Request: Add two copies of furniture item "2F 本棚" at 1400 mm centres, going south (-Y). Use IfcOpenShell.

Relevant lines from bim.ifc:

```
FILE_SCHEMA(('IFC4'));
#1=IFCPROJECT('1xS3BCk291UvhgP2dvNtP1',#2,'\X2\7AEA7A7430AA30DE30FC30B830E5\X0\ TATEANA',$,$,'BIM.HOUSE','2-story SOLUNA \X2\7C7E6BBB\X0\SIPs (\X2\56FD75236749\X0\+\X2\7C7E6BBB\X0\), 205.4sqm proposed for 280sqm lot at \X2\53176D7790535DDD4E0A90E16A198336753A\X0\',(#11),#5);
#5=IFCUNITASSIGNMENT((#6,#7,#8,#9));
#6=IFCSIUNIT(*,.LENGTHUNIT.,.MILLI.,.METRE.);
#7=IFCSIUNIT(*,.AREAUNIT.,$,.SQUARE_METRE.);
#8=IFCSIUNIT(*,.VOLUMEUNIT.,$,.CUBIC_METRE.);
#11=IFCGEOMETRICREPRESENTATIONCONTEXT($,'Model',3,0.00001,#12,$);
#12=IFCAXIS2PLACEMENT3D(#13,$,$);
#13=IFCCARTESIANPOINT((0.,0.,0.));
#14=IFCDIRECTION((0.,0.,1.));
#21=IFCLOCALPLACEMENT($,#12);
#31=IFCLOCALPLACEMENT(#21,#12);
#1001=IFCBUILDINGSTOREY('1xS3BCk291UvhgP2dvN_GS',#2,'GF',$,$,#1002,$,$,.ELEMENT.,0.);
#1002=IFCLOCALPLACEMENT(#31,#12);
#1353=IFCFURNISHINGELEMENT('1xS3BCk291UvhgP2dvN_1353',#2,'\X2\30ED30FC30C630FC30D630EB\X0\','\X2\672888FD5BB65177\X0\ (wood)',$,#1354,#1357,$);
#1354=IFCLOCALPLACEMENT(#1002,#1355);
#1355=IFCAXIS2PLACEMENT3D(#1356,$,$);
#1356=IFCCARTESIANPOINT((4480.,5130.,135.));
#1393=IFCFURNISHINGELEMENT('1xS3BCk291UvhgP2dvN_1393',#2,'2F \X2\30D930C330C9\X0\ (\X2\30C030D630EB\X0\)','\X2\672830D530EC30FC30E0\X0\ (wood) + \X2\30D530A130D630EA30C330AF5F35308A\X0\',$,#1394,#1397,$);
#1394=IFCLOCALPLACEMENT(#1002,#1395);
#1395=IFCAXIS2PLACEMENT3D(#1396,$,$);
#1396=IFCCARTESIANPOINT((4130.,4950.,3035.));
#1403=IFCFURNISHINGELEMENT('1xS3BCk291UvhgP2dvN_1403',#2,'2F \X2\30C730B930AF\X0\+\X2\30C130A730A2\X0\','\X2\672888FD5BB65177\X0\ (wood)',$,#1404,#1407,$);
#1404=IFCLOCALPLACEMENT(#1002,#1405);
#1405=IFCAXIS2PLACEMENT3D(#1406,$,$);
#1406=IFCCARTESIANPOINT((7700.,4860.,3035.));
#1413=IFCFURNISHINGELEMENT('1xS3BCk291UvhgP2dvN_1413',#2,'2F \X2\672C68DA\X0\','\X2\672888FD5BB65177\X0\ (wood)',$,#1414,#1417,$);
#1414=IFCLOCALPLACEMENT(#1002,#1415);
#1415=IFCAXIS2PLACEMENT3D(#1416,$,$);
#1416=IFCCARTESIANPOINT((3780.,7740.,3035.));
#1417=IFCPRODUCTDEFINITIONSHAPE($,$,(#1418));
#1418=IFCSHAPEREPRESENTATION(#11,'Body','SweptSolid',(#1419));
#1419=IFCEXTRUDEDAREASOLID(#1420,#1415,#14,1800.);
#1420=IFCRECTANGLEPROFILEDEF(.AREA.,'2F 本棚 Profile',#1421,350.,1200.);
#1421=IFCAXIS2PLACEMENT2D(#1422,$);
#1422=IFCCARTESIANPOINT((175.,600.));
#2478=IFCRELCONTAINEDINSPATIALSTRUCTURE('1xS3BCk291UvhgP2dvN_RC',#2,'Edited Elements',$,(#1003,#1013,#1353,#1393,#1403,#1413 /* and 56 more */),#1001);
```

```python
import numpy as np
import ifcopenshell
import ifcopenshell.api.geometry
import ifcopenshell.api.root
import ifcopenshell.util.element
import ifcopenshell.util.placement
import ifcopenshell.util.unit

model = ifcopenshell.open("bim.ifc")
unit_scale = ifcopenshell.util.unit.calculate_unit_scale(model)


def reuse_history(source, copy):
    """copy_class also copies each property set's owner history, people and application; keep the originals."""
    for rel in copy.IsDefinedBy:
        if rel.is_a("IfcRelDefinesByProperties") and (history := rel.RelatingPropertyDefinition.OwnerHistory):
            rel.RelatingPropertyDefinition.OwnerHistory = source.OwnerHistory
            ifcopenshell.util.element.remove_deep2(model, history)


source = model.by_guid("1xS3BCk291UvhgP2dvN_1413")
base = ifcopenshell.util.placement.get_local_placement(source.ObjectPlacement)
step = np.array([0.0, -1.0, 0.0]) * 1.4 / unit_scale

for i in range(1, 3):
    copy = ifcopenshell.api.root.copy_class(model, product=source)
    copy.Representation = ifcopenshell.util.element.copy_deep(
        model, source.Representation, exclude=["IfcGeometricRepresentationContext", "IfcRepresentationMap"]
    )
    reuse_history(source, copy)
    matrix = base.copy()
    matrix[:3, 3] += i * step
    print("added at", matrix[:3, 3].round(3) + 0.0)
    ifcopenshell.api.geometry.edit_object_placement(model, product=copy, matrix=matrix, is_si=False)

model.write("bim_v2.ifc")
```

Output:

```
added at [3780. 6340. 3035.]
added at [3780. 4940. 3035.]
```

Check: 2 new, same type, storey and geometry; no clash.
